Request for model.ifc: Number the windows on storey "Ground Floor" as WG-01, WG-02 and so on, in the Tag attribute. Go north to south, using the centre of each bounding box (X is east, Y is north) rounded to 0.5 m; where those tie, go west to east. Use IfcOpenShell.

First a look at what the model holds.

```python
import ifcopenshell
import ifcopenshell.util.element
import ifcopenshell.util.placement

model = ifcopenshell.open("model.ifc")
print(model.schema)
storey = next(s for s in model.by_type("IfcBuildingStorey") if s.Name == "Ground Floor")
windows = [e for e in ifcopenshell.util.element.get_decomposition(storey) if e.is_a("IfcWindow")]
for e in sorted(windows, key=lambda e: e.id()):
    origin = ifcopenshell.util.placement.get_local_placement(e.ObjectPlacement)[:3, 3]
    print(e.id(), e.Tag, e.Name, origin.round(2) + 0.0, sep=" | ")
```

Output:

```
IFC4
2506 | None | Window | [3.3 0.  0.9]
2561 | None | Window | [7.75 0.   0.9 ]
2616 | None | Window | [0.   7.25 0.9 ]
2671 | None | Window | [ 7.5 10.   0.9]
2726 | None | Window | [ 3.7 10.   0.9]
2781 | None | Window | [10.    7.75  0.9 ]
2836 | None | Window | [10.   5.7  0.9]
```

```python
import ifcopenshell
import ifcopenshell.geom
import ifcopenshell.util.element
import ifcopenshell.util.shape

model = ifcopenshell.open("model.ifc")
settings = ifcopenshell.geom.settings()
settings.set("use-world-coords", True)


def centre(element):
    shape = ifcopenshell.geom.create_shape(settings, element)
    return ifcopenshell.util.shape.get_bbox_centroid(shape.geometry)


storey = next(s for s in model.by_type("IfcBuildingStorey") if s.Name == "Ground Floor")
windows = [e for e in ifcopenshell.util.element.get_decomposition(storey) if e.is_a("IfcWindow")]

# Insertion points can sit at a corner or the storey origin, so sort by the geometry (in metres).
centres = {e: centre(e) for e in windows}
windows.sort(key=lambda e: (-round(centres[e][1] / 0.5), centres[e][0]))

for i, e in enumerate(windows, start=1):
    number = f"WG-{i:02d}"
    e.Tag = number
    print(e.id(), number)

model.write("model_v2.ifc")
```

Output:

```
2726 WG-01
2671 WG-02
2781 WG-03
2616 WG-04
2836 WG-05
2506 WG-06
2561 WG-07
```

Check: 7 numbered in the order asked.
